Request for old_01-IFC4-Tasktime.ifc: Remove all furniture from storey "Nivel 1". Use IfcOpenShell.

First a look at what the model holds.

```python
import ifcopenshell
import ifcopenshell.util.element

model = ifcopenshell.open("old_01-IFC4-Tasktime.ifc")
print(model.schema)
storey = next(s for s in model.by_type("IfcBuildingStorey") if s.Name == "Nivel 1")
furniture = [e for e in ifcopenshell.util.element.get_decomposition(storey) if e.is_a("IfcFurnishingElement")]
seen = {}
for e in furniture:
    element_type = ifcopenshell.util.element.get_type(e)
    name = element_type.Name if element_type not in (None, e) else None
    seen[name] = seen.get(name, 0) + 1
for name, count in sorted(seen.items(), key=str):
    print(count, "x", name)
```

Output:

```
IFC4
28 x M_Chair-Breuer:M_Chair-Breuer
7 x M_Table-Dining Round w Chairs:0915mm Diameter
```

```python
import ifcopenshell
import ifcopenshell.api.root
import ifcopenshell.util.element

model = ifcopenshell.open("old_01-IFC4-Tasktime.ifc")

storey = next(s for s in model.by_type("IfcBuildingStorey") if s.Name == "Nivel 1")
furniture = [e for e in ifcopenshell.util.element.get_decomposition(storey) if e.is_a("IfcFurnishingElement")]

for e in furniture:
    ifcopenshell.api.root.remove_product(model, product=e)
print(len(furniture), "removed")

model.write("old_01-IFC4-Tasktime_updated.ifc")
```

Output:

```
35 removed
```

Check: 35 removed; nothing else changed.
